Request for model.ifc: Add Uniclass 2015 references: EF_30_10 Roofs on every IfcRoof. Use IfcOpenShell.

First a look at what the model holds.

```python
import ifcopenshell

model = ifcopenshell.open("model.ifc")
print(model.schema)
print("classifications:", [c.Name for c in model.by_type("IfcClassification")])
for ifc_class in ("IfcDoor", "IfcRoof", "IfcStair", "IfcWall", "IfcWindow"):
    print(ifc_class, len(model.by_type(ifc_class)))
```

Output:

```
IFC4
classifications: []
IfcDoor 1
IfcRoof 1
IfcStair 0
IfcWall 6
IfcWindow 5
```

```python
import ifcopenshell
import ifcopenshell.api.classification

model = ifcopenshell.open("model.ifc")

system = ifcopenshell.api.classification.add_classification(model, classification="Uniclass 2015")

codes = {
    "IfcRoof": ("EF_30_10", "Roofs"),
}
for ifc_class, (code, name) in codes.items():
    products = model.by_type(ifc_class)
    ifcopenshell.api.classification.add_reference(
        model, products=products, classification=system, identification=code, name=name
    )
    print(code, len(products))

model.write("model_rev.ifc")
```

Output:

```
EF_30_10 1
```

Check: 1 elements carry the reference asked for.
